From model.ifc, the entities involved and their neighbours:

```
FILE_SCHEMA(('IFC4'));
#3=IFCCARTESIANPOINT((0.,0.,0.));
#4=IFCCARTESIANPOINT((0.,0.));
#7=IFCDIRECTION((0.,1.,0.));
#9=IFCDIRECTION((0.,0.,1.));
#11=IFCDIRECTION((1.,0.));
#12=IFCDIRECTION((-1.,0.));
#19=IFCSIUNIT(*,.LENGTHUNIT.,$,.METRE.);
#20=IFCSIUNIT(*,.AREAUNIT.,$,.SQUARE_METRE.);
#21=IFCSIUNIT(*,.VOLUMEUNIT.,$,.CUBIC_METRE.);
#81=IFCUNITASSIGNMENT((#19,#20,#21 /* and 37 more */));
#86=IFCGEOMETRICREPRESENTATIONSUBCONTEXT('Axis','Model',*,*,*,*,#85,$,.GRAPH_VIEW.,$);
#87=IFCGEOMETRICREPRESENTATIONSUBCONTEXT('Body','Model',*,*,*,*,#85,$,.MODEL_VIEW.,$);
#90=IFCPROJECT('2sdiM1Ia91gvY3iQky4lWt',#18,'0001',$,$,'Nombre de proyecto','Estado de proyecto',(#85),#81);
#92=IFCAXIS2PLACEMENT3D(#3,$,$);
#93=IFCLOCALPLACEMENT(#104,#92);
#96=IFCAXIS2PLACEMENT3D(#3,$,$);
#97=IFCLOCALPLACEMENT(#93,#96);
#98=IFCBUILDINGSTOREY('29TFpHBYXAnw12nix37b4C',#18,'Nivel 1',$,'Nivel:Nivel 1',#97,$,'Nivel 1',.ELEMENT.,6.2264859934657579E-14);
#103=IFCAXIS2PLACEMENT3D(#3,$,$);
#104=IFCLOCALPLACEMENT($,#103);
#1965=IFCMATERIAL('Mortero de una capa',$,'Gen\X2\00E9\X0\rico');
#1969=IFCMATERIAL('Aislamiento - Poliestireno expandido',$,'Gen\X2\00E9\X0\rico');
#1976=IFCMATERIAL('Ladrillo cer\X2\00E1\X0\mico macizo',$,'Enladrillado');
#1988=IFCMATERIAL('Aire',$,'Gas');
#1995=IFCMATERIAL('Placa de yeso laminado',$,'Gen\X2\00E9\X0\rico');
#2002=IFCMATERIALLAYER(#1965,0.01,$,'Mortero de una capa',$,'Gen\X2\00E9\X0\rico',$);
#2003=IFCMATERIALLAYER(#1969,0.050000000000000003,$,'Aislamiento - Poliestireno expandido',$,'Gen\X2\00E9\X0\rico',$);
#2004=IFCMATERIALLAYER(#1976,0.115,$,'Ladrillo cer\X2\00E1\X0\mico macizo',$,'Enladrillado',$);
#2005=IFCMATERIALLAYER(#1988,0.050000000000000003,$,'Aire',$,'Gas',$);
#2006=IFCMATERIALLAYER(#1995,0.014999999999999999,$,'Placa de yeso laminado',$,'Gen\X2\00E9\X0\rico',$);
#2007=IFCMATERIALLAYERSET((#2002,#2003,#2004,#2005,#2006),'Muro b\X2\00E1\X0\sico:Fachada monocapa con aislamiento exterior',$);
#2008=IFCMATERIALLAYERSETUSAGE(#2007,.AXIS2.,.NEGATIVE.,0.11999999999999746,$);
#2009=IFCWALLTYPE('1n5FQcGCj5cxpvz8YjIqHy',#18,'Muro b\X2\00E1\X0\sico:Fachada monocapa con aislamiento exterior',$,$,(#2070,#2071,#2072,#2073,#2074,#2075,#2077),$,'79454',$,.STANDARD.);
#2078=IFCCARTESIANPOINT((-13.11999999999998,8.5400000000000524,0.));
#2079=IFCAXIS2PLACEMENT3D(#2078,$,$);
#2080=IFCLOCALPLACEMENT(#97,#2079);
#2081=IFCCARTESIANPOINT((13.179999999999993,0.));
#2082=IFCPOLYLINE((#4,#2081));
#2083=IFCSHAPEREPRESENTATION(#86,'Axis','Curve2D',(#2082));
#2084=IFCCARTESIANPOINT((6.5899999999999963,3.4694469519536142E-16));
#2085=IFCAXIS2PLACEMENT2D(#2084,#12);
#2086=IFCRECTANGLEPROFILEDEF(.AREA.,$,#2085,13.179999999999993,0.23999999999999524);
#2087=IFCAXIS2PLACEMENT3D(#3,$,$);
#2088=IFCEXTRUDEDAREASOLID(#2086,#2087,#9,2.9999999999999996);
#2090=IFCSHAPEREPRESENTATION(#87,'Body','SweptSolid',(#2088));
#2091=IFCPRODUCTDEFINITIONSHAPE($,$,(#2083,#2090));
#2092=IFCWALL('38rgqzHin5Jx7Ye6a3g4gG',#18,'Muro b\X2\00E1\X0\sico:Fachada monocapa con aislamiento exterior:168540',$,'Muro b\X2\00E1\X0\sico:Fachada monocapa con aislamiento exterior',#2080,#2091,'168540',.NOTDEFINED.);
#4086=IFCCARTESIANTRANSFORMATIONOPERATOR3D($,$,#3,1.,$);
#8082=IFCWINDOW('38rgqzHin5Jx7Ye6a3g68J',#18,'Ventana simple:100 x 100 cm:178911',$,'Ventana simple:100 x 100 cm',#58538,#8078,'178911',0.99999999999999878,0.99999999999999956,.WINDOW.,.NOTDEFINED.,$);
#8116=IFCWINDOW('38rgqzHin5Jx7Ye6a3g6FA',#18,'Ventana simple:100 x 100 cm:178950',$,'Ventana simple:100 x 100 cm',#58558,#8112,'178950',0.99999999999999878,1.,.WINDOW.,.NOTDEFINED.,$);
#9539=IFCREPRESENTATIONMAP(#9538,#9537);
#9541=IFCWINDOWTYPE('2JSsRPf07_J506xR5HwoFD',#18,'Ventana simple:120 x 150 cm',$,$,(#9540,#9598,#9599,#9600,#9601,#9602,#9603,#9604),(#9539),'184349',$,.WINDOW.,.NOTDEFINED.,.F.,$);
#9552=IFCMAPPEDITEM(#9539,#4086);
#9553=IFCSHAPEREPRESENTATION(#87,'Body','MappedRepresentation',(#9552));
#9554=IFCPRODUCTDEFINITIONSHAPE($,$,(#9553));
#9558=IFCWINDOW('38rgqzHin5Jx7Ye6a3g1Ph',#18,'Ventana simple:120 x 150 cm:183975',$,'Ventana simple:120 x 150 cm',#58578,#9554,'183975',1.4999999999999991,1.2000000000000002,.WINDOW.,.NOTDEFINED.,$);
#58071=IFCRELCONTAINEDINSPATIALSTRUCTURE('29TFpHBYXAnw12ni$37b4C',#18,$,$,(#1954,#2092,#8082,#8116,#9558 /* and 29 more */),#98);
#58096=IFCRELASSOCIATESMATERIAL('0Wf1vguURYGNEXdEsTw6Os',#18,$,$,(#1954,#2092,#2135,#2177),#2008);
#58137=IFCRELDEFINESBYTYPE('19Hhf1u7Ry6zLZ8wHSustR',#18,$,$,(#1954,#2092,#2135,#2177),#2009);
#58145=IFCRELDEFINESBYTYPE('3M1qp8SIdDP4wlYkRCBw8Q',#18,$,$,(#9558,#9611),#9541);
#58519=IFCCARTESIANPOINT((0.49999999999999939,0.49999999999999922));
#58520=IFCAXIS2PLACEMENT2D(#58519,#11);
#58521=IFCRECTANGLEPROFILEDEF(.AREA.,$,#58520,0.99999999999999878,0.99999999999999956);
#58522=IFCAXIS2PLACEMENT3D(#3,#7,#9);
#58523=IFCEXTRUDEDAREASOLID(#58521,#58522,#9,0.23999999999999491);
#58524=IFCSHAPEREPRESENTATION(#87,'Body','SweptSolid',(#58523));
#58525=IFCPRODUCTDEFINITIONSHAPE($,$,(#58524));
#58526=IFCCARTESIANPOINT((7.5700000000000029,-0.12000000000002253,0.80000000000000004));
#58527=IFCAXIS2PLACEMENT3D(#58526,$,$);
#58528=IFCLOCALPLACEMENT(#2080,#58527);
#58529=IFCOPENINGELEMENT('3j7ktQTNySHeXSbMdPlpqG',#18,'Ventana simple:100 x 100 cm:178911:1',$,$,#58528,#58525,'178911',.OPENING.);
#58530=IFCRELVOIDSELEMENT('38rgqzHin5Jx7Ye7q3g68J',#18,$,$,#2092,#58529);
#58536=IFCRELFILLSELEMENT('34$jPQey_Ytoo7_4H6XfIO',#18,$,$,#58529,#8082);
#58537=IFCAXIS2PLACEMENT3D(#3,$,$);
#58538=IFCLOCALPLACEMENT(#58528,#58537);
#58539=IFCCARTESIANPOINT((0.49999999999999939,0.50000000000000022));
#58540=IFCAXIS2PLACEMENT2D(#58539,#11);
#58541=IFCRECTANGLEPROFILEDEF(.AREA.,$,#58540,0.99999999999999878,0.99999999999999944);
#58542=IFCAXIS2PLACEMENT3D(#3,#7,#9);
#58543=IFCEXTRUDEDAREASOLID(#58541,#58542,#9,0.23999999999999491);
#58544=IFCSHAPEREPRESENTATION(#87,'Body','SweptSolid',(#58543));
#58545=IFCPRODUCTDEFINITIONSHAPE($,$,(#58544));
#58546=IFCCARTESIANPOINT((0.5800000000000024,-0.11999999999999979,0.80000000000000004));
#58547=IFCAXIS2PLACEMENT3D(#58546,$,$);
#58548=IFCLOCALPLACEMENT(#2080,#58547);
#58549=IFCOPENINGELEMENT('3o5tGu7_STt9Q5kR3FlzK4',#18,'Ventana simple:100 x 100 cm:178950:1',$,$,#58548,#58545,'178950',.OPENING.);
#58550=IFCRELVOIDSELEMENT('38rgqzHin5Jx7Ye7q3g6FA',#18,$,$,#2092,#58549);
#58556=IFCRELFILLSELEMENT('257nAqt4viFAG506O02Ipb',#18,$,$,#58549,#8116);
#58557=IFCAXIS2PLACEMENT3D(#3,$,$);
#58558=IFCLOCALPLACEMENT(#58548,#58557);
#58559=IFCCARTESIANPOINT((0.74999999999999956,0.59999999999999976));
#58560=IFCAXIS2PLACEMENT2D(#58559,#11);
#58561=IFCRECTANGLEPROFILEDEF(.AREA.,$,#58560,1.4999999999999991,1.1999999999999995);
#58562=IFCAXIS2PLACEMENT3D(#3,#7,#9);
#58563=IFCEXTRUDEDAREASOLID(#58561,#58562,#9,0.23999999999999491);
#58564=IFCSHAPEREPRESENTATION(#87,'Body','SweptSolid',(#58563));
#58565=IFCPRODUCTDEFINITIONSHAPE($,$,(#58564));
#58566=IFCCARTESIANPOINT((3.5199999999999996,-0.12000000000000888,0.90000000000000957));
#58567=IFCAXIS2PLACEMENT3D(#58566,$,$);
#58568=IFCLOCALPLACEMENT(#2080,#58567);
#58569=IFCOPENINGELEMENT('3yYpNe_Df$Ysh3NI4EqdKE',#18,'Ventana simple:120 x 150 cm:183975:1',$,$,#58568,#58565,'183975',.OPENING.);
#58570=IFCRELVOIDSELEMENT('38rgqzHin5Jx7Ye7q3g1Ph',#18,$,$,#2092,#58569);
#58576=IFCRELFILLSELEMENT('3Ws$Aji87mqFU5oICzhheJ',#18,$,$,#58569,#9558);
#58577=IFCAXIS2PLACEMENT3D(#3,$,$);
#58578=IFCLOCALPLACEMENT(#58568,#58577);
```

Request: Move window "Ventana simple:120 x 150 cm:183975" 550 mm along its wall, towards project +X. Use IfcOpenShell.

```python
import ifcopenshell
import ifcopenshell.api.geometry
import ifcopenshell.util.placement
import ifcopenshell.util.unit

model = ifcopenshell.open("model.ifc")
unit_scale = ifcopenshell.util.unit.calculate_unit_scale(model)

window = model.by_guid("38rgqzHin5Jx7Ye6a3g1Ph")
opening = window.FillsVoids[0].RelatingOpeningElement
wall = opening.VoidsElements[0].RelatingBuildingElement

wall_matrix = ifcopenshell.util.placement.get_local_placement(wall.ObjectPlacement)
shift = wall_matrix[:3, 0] * 0.55 / unit_scale
before = ifcopenshell.util.placement.get_local_placement(window.ObjectPlacement)[:3, 3].copy()

# The window is placed relative to its opening, so it follows when the opening moves.
matrix = ifcopenshell.util.placement.get_local_placement(opening.ObjectPlacement)
matrix[:3, 3] += shift
ifcopenshell.api.geometry.edit_object_placement(
    model, product=opening, matrix=matrix, is_si=False, should_transform_children=True
)

after = ifcopenshell.util.placement.get_local_placement(window.ObjectPlacement)[:3, 3]
print("window moved by", (after - before).round(3) + 0.0)

model.write("model_updated.ifc")
```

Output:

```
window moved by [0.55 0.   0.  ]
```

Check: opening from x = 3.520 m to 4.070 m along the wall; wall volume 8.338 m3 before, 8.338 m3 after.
